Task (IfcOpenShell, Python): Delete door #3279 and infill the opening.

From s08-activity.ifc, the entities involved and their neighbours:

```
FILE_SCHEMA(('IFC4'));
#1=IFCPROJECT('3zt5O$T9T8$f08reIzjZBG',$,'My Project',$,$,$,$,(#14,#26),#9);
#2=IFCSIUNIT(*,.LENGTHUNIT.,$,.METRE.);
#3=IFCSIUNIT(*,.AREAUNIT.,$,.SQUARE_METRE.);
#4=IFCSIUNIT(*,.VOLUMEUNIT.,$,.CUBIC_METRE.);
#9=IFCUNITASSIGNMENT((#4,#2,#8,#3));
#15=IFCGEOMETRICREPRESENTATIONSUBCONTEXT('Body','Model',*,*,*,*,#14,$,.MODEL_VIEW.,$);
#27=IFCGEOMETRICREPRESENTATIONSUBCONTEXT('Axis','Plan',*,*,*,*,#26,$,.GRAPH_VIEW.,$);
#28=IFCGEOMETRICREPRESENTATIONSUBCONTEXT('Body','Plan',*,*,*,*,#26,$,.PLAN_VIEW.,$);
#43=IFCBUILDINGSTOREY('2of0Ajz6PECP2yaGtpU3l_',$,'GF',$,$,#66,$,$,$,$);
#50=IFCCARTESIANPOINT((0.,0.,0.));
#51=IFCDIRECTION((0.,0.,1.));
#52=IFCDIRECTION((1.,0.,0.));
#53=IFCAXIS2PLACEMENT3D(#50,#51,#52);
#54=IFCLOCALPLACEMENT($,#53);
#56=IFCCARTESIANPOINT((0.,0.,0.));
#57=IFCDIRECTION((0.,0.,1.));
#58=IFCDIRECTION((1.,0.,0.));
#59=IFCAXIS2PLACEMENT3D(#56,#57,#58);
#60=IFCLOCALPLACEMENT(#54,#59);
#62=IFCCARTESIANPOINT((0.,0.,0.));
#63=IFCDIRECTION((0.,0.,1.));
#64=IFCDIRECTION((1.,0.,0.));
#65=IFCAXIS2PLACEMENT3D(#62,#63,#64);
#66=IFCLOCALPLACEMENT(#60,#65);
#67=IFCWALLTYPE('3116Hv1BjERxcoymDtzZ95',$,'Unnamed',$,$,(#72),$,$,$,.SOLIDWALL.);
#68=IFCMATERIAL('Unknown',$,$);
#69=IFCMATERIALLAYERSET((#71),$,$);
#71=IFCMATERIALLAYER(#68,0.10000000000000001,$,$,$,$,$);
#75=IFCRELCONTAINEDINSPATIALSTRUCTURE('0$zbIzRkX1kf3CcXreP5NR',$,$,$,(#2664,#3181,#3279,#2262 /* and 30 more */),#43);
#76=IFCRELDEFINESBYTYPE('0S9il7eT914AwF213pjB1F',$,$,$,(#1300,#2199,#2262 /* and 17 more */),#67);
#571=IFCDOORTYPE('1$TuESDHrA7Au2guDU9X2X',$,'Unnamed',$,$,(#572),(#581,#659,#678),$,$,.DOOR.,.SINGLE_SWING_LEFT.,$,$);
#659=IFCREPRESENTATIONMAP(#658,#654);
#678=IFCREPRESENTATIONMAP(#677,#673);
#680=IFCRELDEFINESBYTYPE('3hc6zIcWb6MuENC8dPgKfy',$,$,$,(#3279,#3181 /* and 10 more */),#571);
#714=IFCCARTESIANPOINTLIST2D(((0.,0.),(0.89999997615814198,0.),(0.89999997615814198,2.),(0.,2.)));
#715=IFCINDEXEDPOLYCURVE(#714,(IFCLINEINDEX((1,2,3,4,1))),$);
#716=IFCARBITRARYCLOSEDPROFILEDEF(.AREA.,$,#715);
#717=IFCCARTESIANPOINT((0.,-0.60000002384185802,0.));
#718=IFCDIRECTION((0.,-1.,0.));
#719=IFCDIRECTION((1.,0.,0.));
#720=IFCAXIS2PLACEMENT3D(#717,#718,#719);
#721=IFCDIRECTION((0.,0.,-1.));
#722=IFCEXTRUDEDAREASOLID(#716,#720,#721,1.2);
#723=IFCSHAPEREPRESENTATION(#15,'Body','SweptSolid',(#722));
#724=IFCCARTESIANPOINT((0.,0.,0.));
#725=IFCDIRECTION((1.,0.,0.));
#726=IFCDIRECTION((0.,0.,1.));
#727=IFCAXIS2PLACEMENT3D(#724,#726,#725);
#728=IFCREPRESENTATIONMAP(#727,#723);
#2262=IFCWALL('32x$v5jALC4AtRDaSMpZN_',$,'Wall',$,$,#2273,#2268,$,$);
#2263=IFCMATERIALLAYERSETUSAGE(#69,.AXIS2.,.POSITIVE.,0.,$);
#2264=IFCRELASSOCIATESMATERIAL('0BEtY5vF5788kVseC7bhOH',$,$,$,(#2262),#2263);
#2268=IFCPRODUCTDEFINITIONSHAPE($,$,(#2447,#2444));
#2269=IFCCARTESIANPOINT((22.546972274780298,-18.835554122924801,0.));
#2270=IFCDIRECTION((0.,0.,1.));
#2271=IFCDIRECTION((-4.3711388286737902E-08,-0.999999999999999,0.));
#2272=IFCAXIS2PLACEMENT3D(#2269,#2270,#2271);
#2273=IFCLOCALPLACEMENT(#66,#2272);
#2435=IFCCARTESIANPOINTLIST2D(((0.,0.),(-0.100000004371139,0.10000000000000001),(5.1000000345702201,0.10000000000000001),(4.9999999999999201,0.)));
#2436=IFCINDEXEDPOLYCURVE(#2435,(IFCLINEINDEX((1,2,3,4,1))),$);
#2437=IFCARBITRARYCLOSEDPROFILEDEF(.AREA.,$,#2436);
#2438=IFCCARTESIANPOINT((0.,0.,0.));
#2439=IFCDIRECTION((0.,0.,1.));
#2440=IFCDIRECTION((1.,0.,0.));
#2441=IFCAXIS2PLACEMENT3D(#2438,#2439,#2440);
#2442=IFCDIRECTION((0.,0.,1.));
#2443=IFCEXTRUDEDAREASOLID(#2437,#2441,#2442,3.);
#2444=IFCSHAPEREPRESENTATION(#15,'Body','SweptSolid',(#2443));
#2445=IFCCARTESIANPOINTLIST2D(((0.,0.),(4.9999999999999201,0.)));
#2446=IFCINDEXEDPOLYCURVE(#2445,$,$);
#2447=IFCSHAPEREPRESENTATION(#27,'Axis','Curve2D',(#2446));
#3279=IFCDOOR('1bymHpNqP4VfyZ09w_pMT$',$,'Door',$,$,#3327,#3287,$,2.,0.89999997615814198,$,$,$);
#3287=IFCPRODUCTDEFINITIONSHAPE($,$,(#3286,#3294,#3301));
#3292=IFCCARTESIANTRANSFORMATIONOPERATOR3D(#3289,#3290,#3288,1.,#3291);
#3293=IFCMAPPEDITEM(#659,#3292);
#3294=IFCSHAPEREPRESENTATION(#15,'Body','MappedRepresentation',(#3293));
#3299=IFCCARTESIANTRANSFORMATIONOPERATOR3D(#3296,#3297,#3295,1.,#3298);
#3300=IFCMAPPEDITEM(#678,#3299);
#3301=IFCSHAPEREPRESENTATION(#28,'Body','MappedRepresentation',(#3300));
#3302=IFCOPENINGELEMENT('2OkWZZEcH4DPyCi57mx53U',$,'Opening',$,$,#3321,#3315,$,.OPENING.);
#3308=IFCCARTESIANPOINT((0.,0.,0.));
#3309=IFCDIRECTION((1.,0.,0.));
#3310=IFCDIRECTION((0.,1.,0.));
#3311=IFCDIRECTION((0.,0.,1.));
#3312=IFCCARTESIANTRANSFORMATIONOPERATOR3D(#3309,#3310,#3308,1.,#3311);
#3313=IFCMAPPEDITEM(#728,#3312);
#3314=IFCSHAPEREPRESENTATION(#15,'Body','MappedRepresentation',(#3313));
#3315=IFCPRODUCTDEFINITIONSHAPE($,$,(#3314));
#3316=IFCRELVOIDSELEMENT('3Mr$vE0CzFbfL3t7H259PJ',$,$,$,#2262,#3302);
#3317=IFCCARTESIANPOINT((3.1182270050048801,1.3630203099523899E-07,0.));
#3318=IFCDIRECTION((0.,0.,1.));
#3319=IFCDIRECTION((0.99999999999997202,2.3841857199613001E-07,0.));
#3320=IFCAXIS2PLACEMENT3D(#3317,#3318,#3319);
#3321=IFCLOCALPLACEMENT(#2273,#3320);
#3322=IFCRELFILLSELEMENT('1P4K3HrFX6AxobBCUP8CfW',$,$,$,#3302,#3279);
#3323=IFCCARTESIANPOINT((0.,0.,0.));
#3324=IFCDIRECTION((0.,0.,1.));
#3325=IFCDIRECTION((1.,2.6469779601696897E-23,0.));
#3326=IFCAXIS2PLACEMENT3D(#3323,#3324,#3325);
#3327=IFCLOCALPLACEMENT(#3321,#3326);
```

```python
import ifcopenshell
import ifcopenshell.api.feature
import ifcopenshell.api.root
import ifcopenshell.geom
import ifcopenshell.util.shape

model = ifcopenshell.open("s08-activity.ifc")
settings = ifcopenshell.geom.settings()


def volume(element):
    """Net volume in cubic metres, openings subtracted."""
    shape = ifcopenshell.geom.create_shape(settings, element)
    return ifcopenshell.util.shape.get_volume(shape.geometry)


door = model.by_id(3279)
opening = door.FillsVoids[0].RelatingOpeningElement
wall = opening.VoidsElements[0].RelatingBuildingElement
before = volume(wall)

ifcopenshell.api.root.remove_product(model, product=door)
ifcopenshell.api.feature.remove_feature(model, feature=opening)

after = volume(wall)

print(f"wall volume {before:.3f} -> {after:.3f} m3")

model.write("s08-activity_v2.ifc")
```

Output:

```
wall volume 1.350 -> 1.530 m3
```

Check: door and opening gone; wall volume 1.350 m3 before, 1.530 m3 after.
